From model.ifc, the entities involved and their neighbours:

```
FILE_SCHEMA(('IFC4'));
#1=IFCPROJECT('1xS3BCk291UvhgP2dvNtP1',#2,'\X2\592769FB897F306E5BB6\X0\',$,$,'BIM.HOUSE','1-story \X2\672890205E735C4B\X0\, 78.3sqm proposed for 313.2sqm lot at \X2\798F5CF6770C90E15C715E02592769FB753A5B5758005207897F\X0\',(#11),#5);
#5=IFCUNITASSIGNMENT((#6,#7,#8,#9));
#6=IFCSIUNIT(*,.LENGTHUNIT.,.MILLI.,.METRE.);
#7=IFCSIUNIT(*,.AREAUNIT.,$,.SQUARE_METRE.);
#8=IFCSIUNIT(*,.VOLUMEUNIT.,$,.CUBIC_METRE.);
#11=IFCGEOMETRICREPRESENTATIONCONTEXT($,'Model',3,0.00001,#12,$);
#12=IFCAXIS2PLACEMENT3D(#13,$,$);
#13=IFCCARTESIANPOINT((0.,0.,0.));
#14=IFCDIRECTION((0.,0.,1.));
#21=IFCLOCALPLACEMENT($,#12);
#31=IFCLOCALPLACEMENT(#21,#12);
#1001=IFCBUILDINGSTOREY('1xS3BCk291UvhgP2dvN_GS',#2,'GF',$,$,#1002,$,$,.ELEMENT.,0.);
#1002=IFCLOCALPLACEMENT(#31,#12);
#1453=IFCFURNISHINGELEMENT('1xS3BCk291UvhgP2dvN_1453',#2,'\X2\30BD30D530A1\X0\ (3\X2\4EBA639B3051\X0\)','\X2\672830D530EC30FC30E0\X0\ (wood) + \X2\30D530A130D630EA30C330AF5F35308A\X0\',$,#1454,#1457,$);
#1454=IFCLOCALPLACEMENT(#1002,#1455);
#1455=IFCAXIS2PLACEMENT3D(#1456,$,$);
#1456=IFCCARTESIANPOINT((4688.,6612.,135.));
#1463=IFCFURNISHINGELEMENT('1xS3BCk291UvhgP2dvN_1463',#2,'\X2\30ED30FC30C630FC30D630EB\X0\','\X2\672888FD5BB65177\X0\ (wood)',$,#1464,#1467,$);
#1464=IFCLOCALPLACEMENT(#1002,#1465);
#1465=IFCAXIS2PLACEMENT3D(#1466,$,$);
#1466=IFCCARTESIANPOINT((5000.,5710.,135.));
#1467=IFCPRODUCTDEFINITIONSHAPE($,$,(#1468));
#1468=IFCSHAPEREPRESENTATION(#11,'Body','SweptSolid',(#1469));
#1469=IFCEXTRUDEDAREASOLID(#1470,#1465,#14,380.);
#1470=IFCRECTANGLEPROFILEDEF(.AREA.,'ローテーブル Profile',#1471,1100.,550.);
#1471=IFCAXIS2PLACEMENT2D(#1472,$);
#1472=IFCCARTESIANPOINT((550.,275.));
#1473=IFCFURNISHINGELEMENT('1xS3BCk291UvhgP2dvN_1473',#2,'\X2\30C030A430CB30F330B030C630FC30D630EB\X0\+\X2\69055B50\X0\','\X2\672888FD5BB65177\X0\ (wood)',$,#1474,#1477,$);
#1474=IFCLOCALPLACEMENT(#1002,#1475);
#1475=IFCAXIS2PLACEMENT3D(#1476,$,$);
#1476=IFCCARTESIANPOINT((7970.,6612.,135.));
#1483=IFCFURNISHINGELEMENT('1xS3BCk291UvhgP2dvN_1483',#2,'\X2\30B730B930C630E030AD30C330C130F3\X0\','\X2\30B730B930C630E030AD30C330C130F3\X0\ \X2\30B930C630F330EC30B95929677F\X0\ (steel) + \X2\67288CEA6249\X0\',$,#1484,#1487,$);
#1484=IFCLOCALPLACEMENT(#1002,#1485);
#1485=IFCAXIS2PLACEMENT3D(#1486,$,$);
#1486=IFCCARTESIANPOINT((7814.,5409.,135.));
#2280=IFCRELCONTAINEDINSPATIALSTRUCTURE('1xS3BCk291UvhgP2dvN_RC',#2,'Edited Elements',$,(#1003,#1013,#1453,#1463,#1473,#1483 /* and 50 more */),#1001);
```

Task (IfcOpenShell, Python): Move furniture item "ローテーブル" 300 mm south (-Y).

```python
import ifcopenshell
import ifcopenshell.api.geometry
import ifcopenshell.util.placement
import ifcopenshell.util.unit

model = ifcopenshell.open("model.ifc")
unit_scale = ifcopenshell.util.unit.calculate_unit_scale(model)

item = model.by_guid("1xS3BCk291UvhgP2dvN_1463")
matrix = ifcopenshell.util.placement.get_local_placement(item.ObjectPlacement)
matrix[1, 3] -= 0.3 / unit_scale
ifcopenshell.api.geometry.edit_object_placement(model, product=item, matrix=matrix, is_si=False)

print(ifcopenshell.util.placement.get_local_placement(item.ObjectPlacement).round(3) + 0.0)

model.write("model_rev.ifc")
```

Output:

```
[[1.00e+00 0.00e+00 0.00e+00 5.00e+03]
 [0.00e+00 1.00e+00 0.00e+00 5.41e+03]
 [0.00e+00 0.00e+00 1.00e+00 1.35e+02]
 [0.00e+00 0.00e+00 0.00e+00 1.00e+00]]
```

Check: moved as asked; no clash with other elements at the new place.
